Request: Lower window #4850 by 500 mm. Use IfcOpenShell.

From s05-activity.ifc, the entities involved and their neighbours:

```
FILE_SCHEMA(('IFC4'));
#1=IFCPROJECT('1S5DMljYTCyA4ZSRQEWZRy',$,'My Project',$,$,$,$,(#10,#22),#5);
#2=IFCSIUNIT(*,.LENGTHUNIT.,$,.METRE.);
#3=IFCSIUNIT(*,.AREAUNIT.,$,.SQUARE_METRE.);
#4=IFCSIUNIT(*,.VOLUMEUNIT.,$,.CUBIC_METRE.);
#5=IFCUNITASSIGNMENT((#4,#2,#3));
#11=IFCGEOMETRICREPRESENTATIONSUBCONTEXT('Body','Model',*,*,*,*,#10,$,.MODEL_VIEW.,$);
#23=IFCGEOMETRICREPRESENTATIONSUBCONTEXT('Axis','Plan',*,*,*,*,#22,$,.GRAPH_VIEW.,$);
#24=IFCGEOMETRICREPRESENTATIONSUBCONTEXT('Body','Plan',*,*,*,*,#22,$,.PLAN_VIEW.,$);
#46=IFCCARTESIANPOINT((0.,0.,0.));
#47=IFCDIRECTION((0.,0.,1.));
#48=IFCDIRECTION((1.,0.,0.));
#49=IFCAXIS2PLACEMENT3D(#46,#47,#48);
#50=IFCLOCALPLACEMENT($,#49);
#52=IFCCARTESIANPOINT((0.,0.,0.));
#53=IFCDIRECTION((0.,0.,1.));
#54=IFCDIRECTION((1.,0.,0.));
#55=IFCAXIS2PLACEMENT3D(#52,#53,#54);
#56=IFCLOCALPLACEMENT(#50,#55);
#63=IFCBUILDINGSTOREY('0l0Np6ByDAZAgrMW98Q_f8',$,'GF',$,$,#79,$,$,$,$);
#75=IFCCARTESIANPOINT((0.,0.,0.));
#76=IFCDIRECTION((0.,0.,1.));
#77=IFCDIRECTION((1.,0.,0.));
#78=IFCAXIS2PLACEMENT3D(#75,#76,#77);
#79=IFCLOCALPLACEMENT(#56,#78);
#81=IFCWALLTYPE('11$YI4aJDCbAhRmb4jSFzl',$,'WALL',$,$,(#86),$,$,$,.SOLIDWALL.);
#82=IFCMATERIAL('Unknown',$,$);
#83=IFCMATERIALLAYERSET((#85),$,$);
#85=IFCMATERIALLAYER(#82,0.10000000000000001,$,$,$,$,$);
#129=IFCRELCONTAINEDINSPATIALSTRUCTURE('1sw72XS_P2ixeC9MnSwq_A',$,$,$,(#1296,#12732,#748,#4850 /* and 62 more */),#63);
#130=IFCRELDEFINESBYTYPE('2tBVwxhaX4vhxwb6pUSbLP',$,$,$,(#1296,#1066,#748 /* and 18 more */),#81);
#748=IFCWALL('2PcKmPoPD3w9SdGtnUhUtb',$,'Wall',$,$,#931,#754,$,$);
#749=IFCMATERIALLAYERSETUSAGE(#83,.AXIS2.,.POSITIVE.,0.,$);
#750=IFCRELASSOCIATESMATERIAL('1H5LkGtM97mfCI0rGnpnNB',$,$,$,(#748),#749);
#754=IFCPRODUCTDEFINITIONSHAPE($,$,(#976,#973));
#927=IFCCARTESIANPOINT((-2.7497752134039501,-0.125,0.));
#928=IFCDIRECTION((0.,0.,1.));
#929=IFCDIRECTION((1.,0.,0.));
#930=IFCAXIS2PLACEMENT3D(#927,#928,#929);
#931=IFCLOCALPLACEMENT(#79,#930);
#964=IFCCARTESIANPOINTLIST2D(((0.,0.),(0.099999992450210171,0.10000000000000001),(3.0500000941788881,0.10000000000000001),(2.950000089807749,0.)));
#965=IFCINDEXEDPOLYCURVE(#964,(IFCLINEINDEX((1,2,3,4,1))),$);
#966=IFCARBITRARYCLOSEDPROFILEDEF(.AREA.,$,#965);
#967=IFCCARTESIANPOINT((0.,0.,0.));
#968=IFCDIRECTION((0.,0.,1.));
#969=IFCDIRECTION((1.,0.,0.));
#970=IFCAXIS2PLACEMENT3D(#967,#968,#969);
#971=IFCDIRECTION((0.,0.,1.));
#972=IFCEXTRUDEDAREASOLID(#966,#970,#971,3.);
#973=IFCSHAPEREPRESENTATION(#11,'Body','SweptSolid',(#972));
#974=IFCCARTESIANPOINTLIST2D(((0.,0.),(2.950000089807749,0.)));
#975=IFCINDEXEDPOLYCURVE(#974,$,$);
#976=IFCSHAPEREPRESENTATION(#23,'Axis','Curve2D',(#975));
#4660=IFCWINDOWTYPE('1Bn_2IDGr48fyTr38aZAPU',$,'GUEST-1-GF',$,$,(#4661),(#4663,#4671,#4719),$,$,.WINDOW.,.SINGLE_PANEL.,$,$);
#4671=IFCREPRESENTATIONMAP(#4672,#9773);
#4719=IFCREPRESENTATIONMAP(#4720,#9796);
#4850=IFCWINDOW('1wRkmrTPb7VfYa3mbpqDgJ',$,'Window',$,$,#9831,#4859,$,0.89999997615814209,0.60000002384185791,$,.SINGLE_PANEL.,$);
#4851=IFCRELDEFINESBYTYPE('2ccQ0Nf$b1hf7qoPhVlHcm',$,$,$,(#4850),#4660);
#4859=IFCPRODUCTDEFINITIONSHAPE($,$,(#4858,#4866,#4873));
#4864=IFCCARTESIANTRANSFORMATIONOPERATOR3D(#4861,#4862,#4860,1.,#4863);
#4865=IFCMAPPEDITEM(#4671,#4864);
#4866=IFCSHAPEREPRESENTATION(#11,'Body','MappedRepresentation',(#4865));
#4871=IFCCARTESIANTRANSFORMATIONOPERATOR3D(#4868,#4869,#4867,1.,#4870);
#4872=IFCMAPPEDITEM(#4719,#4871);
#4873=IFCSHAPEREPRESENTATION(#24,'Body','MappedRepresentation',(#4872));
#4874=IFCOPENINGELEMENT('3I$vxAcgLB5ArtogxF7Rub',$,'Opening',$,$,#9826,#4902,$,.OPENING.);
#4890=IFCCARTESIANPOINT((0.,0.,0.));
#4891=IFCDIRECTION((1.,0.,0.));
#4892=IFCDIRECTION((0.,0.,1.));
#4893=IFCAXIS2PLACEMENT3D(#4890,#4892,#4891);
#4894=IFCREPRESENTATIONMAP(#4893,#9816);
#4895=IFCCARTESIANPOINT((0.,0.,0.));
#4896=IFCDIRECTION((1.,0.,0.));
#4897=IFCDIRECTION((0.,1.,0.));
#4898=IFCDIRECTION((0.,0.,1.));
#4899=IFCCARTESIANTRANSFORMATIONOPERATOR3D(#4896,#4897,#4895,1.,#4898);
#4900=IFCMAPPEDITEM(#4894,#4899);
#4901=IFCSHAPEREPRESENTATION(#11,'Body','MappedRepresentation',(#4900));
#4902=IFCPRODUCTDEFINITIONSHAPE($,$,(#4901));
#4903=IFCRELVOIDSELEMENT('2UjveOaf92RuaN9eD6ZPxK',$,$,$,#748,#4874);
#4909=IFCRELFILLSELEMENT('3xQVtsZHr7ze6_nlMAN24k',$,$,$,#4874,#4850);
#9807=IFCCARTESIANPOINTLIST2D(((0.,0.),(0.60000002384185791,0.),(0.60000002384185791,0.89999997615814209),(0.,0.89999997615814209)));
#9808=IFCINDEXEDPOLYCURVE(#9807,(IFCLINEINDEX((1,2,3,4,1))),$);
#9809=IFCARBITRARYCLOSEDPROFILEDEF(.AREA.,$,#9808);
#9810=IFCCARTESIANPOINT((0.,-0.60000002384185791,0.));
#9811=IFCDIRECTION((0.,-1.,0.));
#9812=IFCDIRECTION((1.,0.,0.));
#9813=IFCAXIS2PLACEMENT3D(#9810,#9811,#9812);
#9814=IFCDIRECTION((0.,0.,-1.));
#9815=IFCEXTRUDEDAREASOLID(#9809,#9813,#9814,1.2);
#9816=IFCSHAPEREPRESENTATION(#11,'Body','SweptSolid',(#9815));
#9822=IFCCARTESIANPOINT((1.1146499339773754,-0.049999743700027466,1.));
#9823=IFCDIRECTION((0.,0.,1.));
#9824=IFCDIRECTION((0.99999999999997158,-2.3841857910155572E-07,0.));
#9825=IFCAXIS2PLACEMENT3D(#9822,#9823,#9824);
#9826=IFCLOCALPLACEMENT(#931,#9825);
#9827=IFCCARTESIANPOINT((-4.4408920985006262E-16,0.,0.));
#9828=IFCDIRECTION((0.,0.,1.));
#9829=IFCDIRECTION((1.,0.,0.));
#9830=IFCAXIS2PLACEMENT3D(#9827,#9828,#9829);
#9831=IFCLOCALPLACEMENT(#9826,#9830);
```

```python
import numpy as np
import ifcopenshell
import ifcopenshell.api.geometry
import ifcopenshell.util.placement
import ifcopenshell.util.unit

model = ifcopenshell.open("s05-activity.ifc")
unit_scale = ifcopenshell.util.unit.calculate_unit_scale(model)

window = model.by_id(4850)
opening = window.FillsVoids[0].RelatingOpeningElement
dz = -0.5

shift = np.array([0.0, 0.0, dz])
# The window is placed relative to its opening, so it follows when the opening moves.
matrix = ifcopenshell.util.placement.get_local_placement(opening.ObjectPlacement)
matrix[:3, 3] += shift
ifcopenshell.api.geometry.edit_object_placement(
    model, product=opening, matrix=matrix, is_si=False, should_transform_children=True
)

print(f"moved by {dz * unit_scale:+.3f} m")

model.write("s05-activity_v2.ifc")
```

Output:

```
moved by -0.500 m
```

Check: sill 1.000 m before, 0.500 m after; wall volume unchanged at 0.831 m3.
